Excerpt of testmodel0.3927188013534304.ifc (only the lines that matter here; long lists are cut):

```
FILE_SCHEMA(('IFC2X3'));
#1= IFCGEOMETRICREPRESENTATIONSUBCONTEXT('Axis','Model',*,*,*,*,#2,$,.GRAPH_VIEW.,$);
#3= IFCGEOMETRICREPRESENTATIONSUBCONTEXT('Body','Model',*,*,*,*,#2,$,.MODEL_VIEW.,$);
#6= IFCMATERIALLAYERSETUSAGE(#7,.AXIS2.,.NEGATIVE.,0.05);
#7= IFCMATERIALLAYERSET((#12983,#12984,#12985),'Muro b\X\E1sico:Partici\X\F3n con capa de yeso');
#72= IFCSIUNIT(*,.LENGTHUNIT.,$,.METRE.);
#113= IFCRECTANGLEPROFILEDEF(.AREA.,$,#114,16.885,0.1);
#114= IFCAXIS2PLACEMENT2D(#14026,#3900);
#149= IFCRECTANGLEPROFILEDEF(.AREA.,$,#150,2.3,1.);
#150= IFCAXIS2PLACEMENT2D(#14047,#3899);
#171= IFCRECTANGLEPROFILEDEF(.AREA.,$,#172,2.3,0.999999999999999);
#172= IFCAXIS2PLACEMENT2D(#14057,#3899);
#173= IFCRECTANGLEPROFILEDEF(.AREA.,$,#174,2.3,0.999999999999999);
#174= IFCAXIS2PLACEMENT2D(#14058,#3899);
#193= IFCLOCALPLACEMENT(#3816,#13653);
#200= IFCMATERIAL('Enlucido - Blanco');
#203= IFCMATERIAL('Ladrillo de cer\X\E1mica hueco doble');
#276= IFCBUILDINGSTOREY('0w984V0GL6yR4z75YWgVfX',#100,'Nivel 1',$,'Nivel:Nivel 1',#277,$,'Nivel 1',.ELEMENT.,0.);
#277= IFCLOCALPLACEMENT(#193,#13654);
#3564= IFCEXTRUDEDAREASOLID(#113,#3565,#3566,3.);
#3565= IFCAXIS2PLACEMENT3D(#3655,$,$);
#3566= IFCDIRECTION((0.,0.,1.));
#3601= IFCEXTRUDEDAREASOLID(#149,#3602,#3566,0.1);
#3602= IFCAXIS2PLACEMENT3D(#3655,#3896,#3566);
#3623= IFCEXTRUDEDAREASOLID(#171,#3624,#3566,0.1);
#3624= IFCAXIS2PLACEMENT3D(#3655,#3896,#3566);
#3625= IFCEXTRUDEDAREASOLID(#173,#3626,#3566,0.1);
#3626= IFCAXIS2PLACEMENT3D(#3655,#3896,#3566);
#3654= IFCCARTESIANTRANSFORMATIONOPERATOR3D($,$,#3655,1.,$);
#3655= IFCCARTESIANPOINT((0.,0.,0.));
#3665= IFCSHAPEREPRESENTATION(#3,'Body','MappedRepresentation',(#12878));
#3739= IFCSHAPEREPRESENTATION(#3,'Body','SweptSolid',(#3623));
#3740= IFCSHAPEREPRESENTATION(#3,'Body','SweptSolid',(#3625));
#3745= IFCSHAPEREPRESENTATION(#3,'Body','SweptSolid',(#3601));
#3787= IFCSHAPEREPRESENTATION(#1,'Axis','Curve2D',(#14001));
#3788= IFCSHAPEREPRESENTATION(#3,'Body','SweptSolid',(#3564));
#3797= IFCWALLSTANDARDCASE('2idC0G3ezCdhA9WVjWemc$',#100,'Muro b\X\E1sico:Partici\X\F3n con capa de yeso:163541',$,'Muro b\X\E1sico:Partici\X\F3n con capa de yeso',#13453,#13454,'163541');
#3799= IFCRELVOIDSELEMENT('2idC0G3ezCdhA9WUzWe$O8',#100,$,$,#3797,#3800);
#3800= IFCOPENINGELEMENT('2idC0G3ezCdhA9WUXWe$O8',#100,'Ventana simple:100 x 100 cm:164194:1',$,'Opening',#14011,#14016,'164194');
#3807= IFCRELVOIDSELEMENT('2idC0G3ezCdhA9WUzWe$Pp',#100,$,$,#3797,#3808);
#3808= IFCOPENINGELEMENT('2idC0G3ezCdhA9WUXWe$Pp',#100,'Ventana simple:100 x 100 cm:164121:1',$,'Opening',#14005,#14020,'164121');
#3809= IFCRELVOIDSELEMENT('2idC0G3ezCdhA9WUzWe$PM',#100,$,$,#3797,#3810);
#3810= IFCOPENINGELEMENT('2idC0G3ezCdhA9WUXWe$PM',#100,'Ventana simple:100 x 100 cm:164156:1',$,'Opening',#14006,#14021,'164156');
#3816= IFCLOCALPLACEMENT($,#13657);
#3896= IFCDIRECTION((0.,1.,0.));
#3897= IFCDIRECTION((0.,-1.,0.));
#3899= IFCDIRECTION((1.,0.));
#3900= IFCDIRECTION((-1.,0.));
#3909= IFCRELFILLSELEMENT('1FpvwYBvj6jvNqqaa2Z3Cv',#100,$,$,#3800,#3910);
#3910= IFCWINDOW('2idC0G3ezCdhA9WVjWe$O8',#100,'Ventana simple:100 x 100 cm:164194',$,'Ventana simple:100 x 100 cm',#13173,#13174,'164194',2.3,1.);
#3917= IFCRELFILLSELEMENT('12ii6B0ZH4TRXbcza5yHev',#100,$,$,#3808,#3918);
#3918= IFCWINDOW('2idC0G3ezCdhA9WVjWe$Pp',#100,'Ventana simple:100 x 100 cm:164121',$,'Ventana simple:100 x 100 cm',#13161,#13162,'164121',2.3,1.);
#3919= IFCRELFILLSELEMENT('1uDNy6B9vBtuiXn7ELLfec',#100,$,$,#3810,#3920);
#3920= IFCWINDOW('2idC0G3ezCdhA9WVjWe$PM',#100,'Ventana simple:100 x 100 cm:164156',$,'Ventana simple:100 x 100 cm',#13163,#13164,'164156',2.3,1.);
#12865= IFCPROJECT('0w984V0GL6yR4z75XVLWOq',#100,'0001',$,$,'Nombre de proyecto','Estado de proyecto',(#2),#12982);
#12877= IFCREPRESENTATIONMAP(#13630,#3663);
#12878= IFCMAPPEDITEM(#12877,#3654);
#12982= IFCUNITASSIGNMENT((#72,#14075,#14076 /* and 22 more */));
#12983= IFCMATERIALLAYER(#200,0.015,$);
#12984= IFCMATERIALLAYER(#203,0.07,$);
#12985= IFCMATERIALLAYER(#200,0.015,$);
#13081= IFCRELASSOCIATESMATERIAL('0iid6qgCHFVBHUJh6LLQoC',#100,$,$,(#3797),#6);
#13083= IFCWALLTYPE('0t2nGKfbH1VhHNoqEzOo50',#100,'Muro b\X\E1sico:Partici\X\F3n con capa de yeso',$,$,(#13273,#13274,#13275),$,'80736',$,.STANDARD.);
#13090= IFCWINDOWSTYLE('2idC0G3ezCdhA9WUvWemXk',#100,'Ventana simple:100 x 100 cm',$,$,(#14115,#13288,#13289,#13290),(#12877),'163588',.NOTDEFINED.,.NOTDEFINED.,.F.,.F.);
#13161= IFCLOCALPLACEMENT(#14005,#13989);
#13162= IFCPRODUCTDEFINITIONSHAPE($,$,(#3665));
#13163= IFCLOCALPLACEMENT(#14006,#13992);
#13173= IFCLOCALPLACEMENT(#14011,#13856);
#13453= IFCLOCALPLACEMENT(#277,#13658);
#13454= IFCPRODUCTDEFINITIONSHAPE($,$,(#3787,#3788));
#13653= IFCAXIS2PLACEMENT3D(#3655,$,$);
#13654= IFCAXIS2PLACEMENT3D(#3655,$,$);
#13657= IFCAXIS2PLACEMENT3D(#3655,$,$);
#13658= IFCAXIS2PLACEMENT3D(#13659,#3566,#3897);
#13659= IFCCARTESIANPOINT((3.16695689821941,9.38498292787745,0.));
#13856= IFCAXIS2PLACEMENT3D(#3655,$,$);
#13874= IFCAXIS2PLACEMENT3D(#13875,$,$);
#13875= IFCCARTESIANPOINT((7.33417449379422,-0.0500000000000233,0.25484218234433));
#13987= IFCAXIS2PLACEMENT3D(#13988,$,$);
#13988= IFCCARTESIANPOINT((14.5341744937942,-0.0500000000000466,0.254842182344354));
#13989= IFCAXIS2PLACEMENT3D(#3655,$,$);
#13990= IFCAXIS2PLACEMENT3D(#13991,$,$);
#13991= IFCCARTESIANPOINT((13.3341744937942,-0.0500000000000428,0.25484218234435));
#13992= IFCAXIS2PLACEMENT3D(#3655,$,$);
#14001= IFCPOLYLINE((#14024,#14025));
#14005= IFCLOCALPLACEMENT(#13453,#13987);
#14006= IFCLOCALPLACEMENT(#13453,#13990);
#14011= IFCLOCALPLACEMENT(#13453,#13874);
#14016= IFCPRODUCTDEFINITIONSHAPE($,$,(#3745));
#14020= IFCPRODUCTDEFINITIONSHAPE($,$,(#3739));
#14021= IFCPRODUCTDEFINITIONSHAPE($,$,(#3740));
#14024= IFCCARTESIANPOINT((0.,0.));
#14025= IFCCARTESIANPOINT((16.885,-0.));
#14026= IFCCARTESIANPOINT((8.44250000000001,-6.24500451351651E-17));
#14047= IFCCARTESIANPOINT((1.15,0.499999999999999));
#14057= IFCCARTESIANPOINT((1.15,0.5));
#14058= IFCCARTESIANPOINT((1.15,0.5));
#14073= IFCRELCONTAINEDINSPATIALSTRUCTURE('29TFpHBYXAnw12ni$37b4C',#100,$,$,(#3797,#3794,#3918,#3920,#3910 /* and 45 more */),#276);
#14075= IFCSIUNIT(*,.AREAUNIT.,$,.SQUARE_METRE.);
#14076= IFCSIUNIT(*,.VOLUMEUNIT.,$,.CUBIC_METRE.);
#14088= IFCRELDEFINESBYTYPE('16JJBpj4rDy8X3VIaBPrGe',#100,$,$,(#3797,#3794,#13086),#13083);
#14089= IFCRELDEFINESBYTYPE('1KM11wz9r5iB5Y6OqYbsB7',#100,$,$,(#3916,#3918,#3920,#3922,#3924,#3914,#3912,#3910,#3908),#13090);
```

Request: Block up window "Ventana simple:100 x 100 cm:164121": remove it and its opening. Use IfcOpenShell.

```python
import ifcopenshell
import ifcopenshell.api.feature
import ifcopenshell.api.root
import ifcopenshell.geom
import ifcopenshell.util.shape

model = ifcopenshell.open("testmodel0.3927188013534304.ifc")
settings = ifcopenshell.geom.settings()


def volume(element):
    """Net volume in cubic metres, openings subtracted."""
    shape = ifcopenshell.geom.create_shape(settings, element)
    return ifcopenshell.util.shape.get_volume(shape.geometry)


window = model.by_guid("2idC0G3ezCdhA9WVjWe$Pp")
opening = window.FillsVoids[0].RelatingOpeningElement
wall = opening.VoidsElements[0].RelatingBuildingElement
before = volume(wall)

ifcopenshell.api.root.remove_product(model, product=window)
ifcopenshell.api.feature.remove_feature(model, feature=opening)

after = volume(wall)

print(f"wall volume {before:.3f} -> {after:.3f} m3")

model.write("testmodel0.3927188013534304_edited.ifc")
```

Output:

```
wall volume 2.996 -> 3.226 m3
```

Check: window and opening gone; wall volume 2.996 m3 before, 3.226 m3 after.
